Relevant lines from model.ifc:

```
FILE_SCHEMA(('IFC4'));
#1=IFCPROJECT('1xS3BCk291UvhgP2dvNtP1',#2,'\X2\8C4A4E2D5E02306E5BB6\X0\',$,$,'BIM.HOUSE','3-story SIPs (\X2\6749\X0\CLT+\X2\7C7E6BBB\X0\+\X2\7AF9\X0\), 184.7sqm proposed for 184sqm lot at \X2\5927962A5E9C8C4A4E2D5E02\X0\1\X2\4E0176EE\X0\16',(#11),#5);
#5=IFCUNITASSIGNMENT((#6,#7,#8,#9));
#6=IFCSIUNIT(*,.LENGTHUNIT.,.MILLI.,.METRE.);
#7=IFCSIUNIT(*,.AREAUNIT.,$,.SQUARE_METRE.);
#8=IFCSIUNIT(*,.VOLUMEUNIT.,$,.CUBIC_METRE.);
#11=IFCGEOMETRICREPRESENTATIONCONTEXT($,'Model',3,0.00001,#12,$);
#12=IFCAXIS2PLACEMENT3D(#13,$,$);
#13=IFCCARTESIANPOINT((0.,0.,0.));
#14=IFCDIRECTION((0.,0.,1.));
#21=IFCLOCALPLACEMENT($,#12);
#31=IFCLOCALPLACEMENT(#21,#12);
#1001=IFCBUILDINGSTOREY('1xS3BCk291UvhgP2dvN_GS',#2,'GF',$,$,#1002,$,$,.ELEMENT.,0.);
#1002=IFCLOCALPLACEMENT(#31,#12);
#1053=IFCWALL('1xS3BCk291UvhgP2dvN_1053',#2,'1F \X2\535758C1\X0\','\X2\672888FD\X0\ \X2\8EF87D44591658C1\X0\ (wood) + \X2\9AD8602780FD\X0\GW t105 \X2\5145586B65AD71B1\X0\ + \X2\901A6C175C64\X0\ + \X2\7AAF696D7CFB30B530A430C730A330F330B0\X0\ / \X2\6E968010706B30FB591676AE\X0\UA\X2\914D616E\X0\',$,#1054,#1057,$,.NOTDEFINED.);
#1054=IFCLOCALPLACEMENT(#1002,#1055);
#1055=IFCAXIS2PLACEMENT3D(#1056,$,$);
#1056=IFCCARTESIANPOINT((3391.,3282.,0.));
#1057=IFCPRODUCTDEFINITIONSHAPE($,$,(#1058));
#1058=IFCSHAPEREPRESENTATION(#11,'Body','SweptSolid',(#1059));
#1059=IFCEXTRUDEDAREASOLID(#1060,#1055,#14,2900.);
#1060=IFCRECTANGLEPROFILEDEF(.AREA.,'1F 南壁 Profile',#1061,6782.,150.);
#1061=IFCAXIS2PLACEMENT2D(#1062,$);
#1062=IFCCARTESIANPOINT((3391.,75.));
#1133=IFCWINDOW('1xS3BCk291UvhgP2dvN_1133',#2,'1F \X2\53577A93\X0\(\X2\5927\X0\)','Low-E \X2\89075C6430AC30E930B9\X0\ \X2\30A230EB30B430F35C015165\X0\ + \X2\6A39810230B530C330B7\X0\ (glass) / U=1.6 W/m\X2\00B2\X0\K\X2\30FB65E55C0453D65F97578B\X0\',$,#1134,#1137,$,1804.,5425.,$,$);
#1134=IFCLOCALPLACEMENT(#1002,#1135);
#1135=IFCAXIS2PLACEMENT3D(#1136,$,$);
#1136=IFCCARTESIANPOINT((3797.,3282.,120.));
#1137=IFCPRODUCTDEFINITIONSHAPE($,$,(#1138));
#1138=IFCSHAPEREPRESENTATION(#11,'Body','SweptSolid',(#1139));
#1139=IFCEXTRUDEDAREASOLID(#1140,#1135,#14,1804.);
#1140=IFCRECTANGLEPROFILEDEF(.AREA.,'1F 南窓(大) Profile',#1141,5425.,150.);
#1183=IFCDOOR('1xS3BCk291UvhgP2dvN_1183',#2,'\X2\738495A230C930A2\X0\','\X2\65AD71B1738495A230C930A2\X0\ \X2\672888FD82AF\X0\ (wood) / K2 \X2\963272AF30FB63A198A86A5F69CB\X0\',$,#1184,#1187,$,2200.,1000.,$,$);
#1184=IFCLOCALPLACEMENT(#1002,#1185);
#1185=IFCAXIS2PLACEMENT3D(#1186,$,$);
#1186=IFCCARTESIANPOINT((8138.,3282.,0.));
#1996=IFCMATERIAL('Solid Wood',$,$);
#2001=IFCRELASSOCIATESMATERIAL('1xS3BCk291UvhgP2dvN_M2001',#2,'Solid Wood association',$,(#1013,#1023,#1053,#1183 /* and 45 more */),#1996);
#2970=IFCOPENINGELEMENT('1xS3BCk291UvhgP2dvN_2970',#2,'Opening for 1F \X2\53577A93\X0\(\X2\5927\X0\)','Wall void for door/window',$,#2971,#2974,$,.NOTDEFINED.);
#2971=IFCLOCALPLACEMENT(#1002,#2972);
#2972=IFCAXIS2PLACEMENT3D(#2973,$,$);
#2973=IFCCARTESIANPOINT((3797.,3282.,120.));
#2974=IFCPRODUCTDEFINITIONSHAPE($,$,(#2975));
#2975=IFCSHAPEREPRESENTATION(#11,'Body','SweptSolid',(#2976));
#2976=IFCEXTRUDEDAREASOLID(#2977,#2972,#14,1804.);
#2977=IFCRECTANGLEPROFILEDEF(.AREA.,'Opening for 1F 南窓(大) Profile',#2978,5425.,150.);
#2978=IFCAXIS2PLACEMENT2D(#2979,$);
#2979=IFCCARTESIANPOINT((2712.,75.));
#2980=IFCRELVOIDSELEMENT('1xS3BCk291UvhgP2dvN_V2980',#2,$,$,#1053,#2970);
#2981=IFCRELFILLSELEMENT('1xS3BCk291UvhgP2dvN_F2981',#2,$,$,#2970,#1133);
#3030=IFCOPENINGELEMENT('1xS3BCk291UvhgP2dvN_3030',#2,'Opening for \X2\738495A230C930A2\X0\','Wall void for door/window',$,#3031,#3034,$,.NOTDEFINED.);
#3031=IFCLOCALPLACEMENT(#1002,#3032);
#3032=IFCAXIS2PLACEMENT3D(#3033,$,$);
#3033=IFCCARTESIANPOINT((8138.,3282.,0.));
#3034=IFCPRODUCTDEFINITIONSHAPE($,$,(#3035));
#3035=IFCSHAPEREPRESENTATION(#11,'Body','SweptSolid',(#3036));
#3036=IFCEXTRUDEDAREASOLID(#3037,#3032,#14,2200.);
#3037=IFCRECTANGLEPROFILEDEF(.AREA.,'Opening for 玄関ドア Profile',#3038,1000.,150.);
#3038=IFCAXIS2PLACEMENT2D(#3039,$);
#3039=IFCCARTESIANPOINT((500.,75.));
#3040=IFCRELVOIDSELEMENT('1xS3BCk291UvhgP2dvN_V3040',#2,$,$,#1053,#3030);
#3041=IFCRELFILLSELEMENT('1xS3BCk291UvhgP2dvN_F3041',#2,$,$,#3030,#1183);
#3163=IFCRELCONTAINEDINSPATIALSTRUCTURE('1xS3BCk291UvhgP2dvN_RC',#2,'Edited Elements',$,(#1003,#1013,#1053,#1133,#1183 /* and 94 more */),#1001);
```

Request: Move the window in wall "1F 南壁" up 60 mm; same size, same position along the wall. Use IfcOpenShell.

```python
import numpy as np
import ifcopenshell
import ifcopenshell.api.geometry
import ifcopenshell.util.placement
import ifcopenshell.util.unit

model = ifcopenshell.open("model.ifc")
unit_scale = ifcopenshell.util.unit.calculate_unit_scale(model)

window = model.by_id(1133)
opening = window.FillsVoids[0].RelatingOpeningElement
dz = 0.06 / unit_scale

shift = np.array([0.0, 0.0, dz])
# The window is not placed relative to its opening, so move both.
for product in (opening, window):
    matrix = ifcopenshell.util.placement.get_local_placement(product.ObjectPlacement)
    matrix[:3, 3] += shift
    ifcopenshell.api.geometry.edit_object_placement(model, product=product, matrix=matrix, is_si=False)

print(f"moved by {dz * unit_scale:+.3f} m")

model.write("model_v2.ifc")
```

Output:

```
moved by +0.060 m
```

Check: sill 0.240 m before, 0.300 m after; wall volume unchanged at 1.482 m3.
